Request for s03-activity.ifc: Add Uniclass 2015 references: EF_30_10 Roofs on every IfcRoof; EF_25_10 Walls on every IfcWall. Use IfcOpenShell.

First a look at what the model holds.

```python
import ifcopenshell

model = ifcopenshell.open("s03-activity.ifc")
print(model.schema)
print("classifications:", [c.Name for c in model.by_type("IfcClassification")])
for ifc_class in ("IfcDoor", "IfcRoof", "IfcStair", "IfcWall", "IfcWindow"):
    print(ifc_class, len(model.by_type(ifc_class)))
```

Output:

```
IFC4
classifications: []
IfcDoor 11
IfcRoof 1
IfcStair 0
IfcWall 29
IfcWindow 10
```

```python
import ifcopenshell
import ifcopenshell.api.classification

model = ifcopenshell.open("s03-activity.ifc")

system = ifcopenshell.api.classification.add_classification(model, classification="Uniclass 2015")

codes = {
    "IfcRoof": ("EF_30_10", "Roofs"),
    "IfcWall": ("EF_25_10", "Walls"),
}
for ifc_class, (code, name) in codes.items():
    products = model.by_type(ifc_class)
    ifcopenshell.api.classification.add_reference(
        model, products=products, classification=system, identification=code, name=name
    )
    print(code, len(products))

model.write("s03-activity_rev.ifc")
```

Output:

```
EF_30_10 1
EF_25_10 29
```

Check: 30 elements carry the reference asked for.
